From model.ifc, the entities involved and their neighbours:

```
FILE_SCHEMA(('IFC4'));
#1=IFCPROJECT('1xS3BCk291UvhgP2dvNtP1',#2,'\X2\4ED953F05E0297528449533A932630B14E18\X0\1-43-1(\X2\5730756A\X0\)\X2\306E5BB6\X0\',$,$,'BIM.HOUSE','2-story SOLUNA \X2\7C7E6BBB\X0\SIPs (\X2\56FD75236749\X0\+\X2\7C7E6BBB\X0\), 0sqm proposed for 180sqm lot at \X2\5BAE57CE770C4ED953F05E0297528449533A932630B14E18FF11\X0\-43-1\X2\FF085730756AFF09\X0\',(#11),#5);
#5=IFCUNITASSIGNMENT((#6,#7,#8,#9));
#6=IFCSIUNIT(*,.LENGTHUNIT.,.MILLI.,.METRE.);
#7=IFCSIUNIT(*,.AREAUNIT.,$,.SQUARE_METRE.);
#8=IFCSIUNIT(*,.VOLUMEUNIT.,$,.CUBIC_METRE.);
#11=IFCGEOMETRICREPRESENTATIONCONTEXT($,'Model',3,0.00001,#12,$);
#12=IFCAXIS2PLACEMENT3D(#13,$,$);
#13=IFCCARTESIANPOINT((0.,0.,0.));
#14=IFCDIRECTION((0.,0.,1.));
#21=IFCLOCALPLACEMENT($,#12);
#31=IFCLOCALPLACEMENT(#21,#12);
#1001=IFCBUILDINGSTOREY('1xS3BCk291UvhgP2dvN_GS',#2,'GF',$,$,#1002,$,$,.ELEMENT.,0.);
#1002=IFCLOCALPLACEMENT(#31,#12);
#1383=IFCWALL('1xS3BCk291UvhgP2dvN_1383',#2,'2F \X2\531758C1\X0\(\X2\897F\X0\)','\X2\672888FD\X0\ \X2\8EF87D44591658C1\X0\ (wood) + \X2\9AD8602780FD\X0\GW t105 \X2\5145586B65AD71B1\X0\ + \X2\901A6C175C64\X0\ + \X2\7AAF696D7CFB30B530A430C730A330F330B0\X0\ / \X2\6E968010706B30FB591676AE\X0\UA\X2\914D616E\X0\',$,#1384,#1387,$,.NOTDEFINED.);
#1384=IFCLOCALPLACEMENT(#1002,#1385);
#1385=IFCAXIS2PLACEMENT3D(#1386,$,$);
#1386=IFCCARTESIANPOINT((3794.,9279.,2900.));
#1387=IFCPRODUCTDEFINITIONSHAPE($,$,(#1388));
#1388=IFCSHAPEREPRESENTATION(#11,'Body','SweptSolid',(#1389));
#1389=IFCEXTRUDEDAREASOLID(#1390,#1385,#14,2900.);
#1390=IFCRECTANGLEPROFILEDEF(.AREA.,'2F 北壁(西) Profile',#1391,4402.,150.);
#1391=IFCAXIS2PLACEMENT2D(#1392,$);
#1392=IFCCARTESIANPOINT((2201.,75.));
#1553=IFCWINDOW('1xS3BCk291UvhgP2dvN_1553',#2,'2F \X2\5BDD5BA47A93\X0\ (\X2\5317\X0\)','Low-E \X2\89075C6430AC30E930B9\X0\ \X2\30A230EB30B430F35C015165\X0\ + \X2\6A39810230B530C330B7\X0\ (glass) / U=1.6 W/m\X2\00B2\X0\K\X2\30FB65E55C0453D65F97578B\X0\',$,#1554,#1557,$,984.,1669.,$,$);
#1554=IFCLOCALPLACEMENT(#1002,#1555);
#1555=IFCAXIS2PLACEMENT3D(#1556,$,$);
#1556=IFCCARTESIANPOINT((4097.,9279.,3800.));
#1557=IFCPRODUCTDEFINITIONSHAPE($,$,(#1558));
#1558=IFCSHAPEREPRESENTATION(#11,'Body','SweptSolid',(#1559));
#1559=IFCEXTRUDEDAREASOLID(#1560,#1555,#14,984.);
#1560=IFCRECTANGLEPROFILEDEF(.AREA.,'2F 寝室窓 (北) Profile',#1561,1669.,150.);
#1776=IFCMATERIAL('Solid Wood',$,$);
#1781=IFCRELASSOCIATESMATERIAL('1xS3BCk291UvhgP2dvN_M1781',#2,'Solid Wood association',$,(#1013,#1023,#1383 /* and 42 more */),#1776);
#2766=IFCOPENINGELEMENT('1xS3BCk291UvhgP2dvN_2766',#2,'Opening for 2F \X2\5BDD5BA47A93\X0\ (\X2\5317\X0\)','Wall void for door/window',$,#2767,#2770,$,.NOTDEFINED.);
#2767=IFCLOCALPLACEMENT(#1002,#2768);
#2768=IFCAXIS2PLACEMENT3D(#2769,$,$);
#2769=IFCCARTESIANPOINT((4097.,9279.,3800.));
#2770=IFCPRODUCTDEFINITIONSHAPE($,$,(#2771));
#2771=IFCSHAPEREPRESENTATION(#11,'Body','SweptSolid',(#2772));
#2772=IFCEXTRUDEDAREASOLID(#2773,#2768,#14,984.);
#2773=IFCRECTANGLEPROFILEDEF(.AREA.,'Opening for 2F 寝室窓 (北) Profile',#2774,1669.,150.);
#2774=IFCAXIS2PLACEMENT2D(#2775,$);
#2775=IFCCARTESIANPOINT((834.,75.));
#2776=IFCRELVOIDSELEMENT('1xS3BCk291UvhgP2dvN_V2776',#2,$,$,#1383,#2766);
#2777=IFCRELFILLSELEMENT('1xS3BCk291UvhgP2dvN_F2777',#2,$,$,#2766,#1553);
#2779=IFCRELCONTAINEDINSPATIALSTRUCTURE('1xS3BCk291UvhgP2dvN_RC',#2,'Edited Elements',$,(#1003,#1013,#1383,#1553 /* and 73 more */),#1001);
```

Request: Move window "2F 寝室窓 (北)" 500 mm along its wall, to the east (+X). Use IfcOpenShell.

```python
import ifcopenshell
import ifcopenshell.api.geometry
import ifcopenshell.util.placement

model = ifcopenshell.open("model.ifc")

window = model.by_guid("1xS3BCk291UvhgP2dvN_1553")
opening = window.FillsVoids[0].RelatingOpeningElement
wall = opening.VoidsElements[0].RelatingBuildingElement

wall_matrix = ifcopenshell.util.placement.get_local_placement(wall.ObjectPlacement)
shift = wall_matrix[:3, 0] * 500.0
before = ifcopenshell.util.placement.get_local_placement(window.ObjectPlacement)[:3, 3].copy()

# The window is not placed relative to its opening, so move both.
for product in (opening, window):
    matrix = ifcopenshell.util.placement.get_local_placement(product.ObjectPlacement)
    matrix[:3, 3] += shift
    ifcopenshell.api.geometry.edit_object_placement(model, product=product, matrix=matrix, is_si=False)

after = ifcopenshell.util.placement.get_local_placement(window.ObjectPlacement)[:3, 3]
print("window moved by", (after - before).round(3) + 0.0)

model.write("model_edited.ifc")
```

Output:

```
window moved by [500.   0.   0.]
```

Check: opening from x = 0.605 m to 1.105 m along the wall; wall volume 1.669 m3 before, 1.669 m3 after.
